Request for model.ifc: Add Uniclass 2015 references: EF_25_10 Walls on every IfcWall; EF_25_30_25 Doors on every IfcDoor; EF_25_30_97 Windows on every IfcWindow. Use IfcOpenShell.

First a look at what the model holds.

```python
import ifcopenshell

model = ifcopenshell.open("model.ifc")
print(model.schema)
print("classifications:", [c.Name for c in model.by_type("IfcClassification")])
for ifc_class in ("IfcDoor", "IfcRoof", "IfcStair", "IfcWall", "IfcWindow"):
    print(ifc_class, len(model.by_type(ifc_class)))
```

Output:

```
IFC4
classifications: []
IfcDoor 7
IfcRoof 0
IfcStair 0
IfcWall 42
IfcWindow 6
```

```python
import ifcopenshell
import ifcopenshell.api.classification

model = ifcopenshell.open("model.ifc")

system = ifcopenshell.api.classification.add_classification(model, classification="Uniclass 2015")

codes = {
    "IfcWall": ("EF_25_10", "Walls"),
    "IfcDoor": ("EF_25_30_25", "Doors"),
    "IfcWindow": ("EF_25_30_97", "Windows"),
}
for ifc_class, (code, name) in codes.items():
    products = model.by_type(ifc_class)
    ifcopenshell.api.classification.add_reference(
        model, products=products, classification=system, identification=code, name=name
    )
    print(code, len(products))

model.write("model_v2.ifc")
```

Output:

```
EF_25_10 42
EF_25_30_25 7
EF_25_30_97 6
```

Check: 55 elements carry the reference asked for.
